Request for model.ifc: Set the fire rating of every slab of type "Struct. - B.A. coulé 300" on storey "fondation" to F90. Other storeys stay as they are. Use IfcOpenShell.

First a look at what the model holds.

```python
import ifcopenshell
import ifcopenshell.util.element

model = ifcopenshell.open("model.ifc")
print(model.schema)
storey = next(s for s in model.by_type("IfcBuildingStorey") if s.Name == "fondation")
slabs = [e for e in ifcopenshell.util.element.get_decomposition(storey) if e.is_a("IfcSlab")]
seen = {}
for e in slabs:
    element_type = ifcopenshell.util.element.get_type(e)
    key = (element_type.Name if element_type != e and element_type else None, ifcopenshell.util.element.get_pset(e, "Pset_SlabCommon", "FireRating"))
    seen[key] = seen.get(key, 0) + 1
for (name, value), count in sorted(seen.items(), key=str):
    print(count, "x", name, "|", value)
```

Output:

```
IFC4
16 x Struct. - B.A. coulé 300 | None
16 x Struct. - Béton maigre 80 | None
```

```python
import ifcopenshell
import ifcopenshell.api.pset
import ifcopenshell.util.element

model = ifcopenshell.open("model.ifc")

storey = next(s for s in model.by_type("IfcBuildingStorey") if s.Name == "fondation")
slabs = [e for e in ifcopenshell.util.element.get_decomposition(storey) if e.is_a("IfcSlab")]

count = 0
for e in slabs:
    element_type = ifcopenshell.util.element.get_type(e)
    if element_type in (None, e) or element_type.Name != "Struct. - B.A. coulé 300":
        continue
    # add_pset returns the element's existing set when there is one.
    pset = ifcopenshell.api.pset.add_pset(model, product=e, name="Pset_SlabCommon")
    ifcopenshell.api.pset.edit_pset(model, pset=pset, properties={"FireRating": "F90"})
    count += 1

print(count, "slabs updated")

model.write("model_edited.ifc")
```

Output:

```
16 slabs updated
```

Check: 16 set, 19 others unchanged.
